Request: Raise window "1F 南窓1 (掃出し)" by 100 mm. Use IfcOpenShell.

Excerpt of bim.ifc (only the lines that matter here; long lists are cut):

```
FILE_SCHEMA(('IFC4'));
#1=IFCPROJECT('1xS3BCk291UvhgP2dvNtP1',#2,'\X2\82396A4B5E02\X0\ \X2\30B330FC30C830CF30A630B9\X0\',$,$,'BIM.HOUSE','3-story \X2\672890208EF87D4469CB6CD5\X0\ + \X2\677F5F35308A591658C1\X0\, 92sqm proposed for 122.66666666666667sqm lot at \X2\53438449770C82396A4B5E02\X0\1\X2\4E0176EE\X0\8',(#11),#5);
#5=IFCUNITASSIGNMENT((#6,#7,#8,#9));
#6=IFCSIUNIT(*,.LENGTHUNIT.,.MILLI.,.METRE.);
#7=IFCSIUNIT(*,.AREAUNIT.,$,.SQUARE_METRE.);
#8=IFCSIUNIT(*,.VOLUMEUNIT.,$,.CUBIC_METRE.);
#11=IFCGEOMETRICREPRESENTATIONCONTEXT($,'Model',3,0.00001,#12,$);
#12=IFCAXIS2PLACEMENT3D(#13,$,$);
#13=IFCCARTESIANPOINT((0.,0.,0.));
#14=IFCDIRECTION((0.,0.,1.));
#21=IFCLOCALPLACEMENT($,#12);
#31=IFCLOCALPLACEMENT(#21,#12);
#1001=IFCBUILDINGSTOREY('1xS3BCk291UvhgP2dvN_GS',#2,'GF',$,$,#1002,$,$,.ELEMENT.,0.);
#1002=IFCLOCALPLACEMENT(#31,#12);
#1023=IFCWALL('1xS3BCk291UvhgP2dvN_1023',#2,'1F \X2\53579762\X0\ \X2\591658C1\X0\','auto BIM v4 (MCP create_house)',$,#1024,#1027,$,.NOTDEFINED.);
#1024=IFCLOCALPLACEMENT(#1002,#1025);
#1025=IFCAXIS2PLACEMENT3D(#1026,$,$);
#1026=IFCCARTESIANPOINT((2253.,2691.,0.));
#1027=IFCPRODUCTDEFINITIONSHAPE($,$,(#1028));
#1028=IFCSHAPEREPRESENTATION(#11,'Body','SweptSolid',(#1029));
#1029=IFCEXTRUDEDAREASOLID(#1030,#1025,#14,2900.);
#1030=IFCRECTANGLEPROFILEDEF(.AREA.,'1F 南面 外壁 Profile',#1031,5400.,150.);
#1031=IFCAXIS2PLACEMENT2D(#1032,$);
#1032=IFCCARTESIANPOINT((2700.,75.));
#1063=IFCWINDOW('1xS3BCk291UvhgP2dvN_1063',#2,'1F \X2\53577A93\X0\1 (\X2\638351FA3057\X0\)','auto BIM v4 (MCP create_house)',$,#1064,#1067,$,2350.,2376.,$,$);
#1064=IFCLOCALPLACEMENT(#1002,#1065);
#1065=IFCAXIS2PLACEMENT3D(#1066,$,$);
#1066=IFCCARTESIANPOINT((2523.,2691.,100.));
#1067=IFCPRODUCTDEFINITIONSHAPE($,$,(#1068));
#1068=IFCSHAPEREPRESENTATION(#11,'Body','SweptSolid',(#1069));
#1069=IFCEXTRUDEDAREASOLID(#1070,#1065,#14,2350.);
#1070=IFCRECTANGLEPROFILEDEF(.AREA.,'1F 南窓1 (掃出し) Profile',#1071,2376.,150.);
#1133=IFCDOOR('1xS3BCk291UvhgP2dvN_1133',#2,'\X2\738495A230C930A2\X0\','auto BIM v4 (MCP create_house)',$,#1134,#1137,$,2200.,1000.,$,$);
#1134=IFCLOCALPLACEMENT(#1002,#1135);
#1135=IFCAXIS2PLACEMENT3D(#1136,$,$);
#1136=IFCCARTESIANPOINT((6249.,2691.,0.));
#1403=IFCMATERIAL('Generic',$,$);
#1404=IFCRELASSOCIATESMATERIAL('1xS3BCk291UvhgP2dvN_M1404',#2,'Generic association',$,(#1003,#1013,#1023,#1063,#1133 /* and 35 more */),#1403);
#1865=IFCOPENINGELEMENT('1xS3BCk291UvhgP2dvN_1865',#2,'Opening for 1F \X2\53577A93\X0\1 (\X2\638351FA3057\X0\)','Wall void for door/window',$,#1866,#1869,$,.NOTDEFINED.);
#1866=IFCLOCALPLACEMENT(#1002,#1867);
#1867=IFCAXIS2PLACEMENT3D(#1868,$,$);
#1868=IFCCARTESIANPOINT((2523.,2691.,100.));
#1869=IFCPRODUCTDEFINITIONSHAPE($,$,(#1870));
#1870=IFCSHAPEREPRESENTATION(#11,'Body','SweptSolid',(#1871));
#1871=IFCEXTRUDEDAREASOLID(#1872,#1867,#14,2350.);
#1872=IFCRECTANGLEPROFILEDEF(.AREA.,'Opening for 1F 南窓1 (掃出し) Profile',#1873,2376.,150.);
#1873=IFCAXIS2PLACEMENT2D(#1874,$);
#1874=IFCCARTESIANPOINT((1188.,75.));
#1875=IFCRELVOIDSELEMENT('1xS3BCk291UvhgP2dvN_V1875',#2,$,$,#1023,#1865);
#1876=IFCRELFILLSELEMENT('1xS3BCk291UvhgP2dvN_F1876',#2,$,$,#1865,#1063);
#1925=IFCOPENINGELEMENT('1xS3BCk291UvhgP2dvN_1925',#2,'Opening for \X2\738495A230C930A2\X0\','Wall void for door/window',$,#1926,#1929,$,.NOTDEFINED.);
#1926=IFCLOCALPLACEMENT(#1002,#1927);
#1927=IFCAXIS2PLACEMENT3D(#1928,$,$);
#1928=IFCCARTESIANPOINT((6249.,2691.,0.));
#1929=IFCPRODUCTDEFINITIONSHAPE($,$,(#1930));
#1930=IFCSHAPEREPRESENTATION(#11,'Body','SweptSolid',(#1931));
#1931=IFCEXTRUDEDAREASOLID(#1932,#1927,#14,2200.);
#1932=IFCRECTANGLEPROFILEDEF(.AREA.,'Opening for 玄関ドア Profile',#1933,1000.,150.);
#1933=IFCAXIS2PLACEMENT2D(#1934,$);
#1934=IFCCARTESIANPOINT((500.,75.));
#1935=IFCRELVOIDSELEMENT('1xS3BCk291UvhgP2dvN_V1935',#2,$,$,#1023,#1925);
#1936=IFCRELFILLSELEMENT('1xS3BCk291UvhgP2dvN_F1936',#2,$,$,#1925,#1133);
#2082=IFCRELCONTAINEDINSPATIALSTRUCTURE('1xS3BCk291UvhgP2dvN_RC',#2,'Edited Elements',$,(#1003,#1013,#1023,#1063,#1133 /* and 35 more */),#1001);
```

```python
import numpy as np
import ifcopenshell
import ifcopenshell.api.geometry
import ifcopenshell.util.placement
import ifcopenshell.util.unit

model = ifcopenshell.open("bim.ifc")
unit_scale = ifcopenshell.util.unit.calculate_unit_scale(model)

window = model.by_id(1063)
opening = window.FillsVoids[0].RelatingOpeningElement
dz = 100.0

shift = np.array([0.0, 0.0, dz])
# The window is not placed relative to its opening, so move both.
for product in (opening, window):
    matrix = ifcopenshell.util.placement.get_local_placement(product.ObjectPlacement)
    matrix[:3, 3] += shift
    ifcopenshell.api.geometry.edit_object_placement(model, product=product, matrix=matrix, is_si=False)

print(f"moved by {dz * unit_scale:+.3f} m")

model.write("bim_updated.ifc")
```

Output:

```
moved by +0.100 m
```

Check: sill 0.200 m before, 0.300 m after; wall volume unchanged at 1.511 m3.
